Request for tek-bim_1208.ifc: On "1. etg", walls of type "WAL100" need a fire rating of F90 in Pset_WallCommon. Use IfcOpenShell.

First a look at what the model holds.

```python
import ifcopenshell
import ifcopenshell.util.element

model = ifcopenshell.open("tek-bim_1208.ifc")
print(model.schema)
storey = next(s for s in model.by_type("IfcBuildingStorey") if s.Name == "1. etg")
walls = [e for e in ifcopenshell.util.element.get_decomposition(storey) if e.is_a("IfcWall")]
seen = {}
for e in walls:
    element_type = ifcopenshell.util.element.get_type(e)
    key = (element_type.Name if element_type != e and element_type else None, ifcopenshell.util.element.get_pset(e, "Pset_WallCommon", "FireRating"))
    seen[key] = seen.get(key, 0) + 1
for (name, value), count in sorted(seen.items(), key=str):
    print(count, "x", name, "|", value)
```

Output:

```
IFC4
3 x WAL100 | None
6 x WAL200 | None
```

```python
import ifcopenshell
import ifcopenshell.api.pset
import ifcopenshell.util.element

model = ifcopenshell.open("tek-bim_1208.ifc")

storey = next(s for s in model.by_type("IfcBuildingStorey") if s.Name == "1. etg")
walls = [e for e in ifcopenshell.util.element.get_decomposition(storey) if e.is_a("IfcWall")]

count = 0
for e in walls:
    element_type = ifcopenshell.util.element.get_type(e)
    if element_type in (None, e) or element_type.Name != "WAL100":
        continue
    # add_pset returns the element's existing set when there is one.
    pset = ifcopenshell.api.pset.add_pset(model, product=e, name="Pset_WallCommon")
    ifcopenshell.api.pset.edit_pset(model, pset=pset, properties={"FireRating": "F90"})
    count += 1

print(count, "walls updated")

model.write("tek-bim_1208_v2.ifc")
```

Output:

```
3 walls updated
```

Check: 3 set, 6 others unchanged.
